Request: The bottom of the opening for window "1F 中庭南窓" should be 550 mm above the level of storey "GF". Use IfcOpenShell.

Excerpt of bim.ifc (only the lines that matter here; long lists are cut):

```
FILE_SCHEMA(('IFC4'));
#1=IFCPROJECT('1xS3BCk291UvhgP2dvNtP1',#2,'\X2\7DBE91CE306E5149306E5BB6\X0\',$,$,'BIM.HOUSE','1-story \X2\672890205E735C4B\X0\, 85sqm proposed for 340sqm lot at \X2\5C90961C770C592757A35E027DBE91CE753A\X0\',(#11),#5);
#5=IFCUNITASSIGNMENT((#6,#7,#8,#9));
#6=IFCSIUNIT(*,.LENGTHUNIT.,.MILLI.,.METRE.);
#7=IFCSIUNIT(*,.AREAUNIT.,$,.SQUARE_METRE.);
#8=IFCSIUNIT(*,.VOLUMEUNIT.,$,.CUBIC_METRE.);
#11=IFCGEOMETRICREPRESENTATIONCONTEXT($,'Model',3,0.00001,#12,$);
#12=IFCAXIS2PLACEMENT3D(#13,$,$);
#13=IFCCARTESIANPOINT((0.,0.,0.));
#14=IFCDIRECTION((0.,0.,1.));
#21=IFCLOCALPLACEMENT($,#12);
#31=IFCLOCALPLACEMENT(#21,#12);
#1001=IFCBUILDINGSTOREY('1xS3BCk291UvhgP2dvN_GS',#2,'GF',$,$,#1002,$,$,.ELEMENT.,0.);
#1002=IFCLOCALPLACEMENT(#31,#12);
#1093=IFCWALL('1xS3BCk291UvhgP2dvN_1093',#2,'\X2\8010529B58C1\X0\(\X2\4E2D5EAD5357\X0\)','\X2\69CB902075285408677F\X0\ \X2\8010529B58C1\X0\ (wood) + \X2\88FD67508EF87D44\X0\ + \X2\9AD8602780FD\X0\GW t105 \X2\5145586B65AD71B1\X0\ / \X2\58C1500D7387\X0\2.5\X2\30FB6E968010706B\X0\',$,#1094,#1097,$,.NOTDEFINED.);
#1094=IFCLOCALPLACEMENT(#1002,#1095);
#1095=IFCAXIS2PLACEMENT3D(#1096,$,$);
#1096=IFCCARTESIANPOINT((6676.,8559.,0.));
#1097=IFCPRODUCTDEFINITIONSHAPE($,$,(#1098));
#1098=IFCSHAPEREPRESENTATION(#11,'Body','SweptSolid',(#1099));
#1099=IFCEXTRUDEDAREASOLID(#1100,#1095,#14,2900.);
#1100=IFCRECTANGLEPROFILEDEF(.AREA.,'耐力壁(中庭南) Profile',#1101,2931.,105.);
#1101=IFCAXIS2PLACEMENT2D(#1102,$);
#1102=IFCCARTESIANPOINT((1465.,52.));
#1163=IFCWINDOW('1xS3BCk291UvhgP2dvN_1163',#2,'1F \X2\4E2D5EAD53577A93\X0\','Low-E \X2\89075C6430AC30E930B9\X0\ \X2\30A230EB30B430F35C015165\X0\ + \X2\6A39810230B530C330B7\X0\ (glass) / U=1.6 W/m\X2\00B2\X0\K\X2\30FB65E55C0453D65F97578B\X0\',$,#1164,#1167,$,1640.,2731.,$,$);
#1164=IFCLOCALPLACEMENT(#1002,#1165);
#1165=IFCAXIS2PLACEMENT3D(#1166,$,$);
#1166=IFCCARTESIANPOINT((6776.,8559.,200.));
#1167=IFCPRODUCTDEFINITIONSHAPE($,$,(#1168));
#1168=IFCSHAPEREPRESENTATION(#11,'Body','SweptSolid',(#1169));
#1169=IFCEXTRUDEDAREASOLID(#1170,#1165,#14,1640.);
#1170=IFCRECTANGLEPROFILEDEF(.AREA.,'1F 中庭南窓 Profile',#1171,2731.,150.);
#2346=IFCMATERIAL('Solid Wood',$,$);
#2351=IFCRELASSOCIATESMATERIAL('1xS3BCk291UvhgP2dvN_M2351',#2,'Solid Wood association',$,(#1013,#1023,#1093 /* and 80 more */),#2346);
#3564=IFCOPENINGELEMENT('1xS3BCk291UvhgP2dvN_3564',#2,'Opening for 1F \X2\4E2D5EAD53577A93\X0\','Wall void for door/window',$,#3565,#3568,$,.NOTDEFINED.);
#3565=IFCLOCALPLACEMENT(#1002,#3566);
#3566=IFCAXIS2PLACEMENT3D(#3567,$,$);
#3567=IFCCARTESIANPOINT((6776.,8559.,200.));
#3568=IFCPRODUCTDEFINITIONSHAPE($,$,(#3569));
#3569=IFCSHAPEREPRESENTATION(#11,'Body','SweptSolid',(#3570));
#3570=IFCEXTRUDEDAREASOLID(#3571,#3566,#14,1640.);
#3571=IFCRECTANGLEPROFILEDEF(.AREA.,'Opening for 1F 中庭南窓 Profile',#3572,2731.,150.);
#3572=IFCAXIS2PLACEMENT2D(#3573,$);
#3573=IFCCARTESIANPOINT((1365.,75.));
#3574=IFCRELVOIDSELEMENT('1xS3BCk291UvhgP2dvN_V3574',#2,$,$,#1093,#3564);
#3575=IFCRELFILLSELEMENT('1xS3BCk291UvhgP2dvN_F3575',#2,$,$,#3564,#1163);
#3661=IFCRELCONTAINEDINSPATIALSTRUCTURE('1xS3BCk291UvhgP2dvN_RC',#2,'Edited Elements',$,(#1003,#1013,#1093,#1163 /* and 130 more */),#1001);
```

```python
import numpy as np
import ifcopenshell
import ifcopenshell.api.geometry
import ifcopenshell.geom
import ifcopenshell.util.element
import ifcopenshell.util.placement
import ifcopenshell.util.shape
import ifcopenshell.util.unit

model = ifcopenshell.open("bim.ifc")
unit_scale = ifcopenshell.util.unit.calculate_unit_scale(model)

window = model.by_guid("1xS3BCk291UvhgP2dvN_1163")
opening = window.FillsVoids[0].RelatingOpeningElement
storey = ifcopenshell.util.element.get_container(window, ifc_class="IfcBuildingStorey")
level = ifcopenshell.util.placement.get_local_placement(storey.ObjectPlacement)[2, 3]

# The opening's origin need not be at the sill, so measure its lowest point.
shape = ifcopenshell.geom.create_shape(ifcopenshell.geom.settings(), opening)
bottom = ifcopenshell.util.shape.get_shape_bottom_elevation(shape, shape.geometry) / unit_scale
dz = level + 0.55 / unit_scale - bottom

shift = np.array([0.0, 0.0, dz])
# The window is not placed relative to its opening, so move both.
for product in (opening, window):
    matrix = ifcopenshell.util.placement.get_local_placement(product.ObjectPlacement)
    matrix[:3, 3] += shift
    ifcopenshell.api.geometry.edit_object_placement(model, product=product, matrix=matrix, is_si=False)

print(f"moved by {dz * unit_scale:+.3f} m")

model.write("bim_updated.ifc")
```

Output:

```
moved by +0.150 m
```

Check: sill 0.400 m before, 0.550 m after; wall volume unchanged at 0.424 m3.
